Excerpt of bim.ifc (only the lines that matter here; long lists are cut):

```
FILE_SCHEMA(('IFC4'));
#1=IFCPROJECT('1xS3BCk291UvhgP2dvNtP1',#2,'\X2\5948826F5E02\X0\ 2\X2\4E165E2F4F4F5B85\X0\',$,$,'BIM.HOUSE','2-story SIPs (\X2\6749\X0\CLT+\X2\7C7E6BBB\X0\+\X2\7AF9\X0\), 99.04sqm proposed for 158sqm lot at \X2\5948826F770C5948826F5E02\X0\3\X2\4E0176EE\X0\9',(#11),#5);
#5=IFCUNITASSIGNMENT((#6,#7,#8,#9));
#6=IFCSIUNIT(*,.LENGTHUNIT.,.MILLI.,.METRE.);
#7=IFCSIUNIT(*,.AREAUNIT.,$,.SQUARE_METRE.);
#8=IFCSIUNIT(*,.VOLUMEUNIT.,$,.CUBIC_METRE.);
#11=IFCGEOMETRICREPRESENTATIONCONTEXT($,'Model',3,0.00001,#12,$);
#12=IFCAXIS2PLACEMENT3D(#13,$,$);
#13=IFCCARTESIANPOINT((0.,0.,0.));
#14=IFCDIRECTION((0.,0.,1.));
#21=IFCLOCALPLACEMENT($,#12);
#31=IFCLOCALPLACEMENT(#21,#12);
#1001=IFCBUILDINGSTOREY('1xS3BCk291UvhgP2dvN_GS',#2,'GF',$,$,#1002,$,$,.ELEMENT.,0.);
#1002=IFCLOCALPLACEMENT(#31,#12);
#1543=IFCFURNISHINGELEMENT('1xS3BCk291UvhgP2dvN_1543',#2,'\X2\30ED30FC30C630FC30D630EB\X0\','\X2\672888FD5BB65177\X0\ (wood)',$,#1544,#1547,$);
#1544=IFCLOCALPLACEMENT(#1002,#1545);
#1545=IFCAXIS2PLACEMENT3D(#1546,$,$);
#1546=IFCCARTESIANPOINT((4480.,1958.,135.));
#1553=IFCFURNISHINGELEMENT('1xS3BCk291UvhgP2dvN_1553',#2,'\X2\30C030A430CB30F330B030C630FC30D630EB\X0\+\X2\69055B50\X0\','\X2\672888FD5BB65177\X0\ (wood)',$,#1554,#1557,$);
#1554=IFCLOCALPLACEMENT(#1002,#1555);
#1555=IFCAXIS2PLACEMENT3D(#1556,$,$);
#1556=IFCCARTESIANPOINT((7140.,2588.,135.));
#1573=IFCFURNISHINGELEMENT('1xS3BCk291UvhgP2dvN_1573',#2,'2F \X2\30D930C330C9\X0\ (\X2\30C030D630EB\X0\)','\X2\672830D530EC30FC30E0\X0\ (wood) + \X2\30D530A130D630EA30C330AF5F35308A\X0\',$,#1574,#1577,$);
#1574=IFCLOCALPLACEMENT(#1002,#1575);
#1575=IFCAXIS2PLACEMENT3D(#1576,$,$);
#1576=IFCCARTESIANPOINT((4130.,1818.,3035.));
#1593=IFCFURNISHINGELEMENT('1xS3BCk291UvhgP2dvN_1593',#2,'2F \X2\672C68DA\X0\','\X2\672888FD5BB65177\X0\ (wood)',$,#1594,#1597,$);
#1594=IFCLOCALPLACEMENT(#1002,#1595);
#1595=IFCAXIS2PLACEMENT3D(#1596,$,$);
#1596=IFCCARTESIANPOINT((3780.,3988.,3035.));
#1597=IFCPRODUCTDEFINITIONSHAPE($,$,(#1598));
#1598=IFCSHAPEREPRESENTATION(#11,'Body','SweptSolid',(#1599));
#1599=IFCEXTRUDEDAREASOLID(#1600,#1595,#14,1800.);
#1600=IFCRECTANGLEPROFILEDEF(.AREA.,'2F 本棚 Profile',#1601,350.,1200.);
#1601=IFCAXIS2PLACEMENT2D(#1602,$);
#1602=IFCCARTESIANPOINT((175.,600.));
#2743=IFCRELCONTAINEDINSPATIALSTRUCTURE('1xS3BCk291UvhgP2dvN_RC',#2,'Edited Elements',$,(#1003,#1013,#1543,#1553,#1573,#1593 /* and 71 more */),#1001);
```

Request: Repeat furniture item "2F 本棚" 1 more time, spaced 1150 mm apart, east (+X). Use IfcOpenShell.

```python
import numpy as np
import ifcopenshell
import ifcopenshell.api.geometry
import ifcopenshell.api.root
import ifcopenshell.util.element
import ifcopenshell.util.placement
import ifcopenshell.util.unit

model = ifcopenshell.open("bim.ifc")
unit_scale = ifcopenshell.util.unit.calculate_unit_scale(model)


def reuse_history(source, copy):
    """copy_class also copies each property set's owner history, people and application; keep the originals."""
    for rel in copy.IsDefinedBy:
        if rel.is_a("IfcRelDefinesByProperties") and (history := rel.RelatingPropertyDefinition.OwnerHistory):
            rel.RelatingPropertyDefinition.OwnerHistory = source.OwnerHistory
            ifcopenshell.util.element.remove_deep2(model, history)


source = model.by_guid("1xS3BCk291UvhgP2dvN_1593")
base = ifcopenshell.util.placement.get_local_placement(source.ObjectPlacement)
step = np.array([1.0, 0.0, 0.0]) * 1.15 / unit_scale

for i in range(1, 2):
    copy = ifcopenshell.api.root.copy_class(model, product=source)
    copy.Representation = ifcopenshell.util.element.copy_deep(
        model, source.Representation, exclude=["IfcGeometricRepresentationContext", "IfcRepresentationMap"]
    )
    reuse_history(source, copy)
    matrix = base.copy()
    matrix[:3, 3] += i * step
    print("added at", matrix[:3, 3].round(3) + 0.0)
    ifcopenshell.api.geometry.edit_object_placement(model, product=copy, matrix=matrix, is_si=False)

model.write("bim_edited.ifc")
```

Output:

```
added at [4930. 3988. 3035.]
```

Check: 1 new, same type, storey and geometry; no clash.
